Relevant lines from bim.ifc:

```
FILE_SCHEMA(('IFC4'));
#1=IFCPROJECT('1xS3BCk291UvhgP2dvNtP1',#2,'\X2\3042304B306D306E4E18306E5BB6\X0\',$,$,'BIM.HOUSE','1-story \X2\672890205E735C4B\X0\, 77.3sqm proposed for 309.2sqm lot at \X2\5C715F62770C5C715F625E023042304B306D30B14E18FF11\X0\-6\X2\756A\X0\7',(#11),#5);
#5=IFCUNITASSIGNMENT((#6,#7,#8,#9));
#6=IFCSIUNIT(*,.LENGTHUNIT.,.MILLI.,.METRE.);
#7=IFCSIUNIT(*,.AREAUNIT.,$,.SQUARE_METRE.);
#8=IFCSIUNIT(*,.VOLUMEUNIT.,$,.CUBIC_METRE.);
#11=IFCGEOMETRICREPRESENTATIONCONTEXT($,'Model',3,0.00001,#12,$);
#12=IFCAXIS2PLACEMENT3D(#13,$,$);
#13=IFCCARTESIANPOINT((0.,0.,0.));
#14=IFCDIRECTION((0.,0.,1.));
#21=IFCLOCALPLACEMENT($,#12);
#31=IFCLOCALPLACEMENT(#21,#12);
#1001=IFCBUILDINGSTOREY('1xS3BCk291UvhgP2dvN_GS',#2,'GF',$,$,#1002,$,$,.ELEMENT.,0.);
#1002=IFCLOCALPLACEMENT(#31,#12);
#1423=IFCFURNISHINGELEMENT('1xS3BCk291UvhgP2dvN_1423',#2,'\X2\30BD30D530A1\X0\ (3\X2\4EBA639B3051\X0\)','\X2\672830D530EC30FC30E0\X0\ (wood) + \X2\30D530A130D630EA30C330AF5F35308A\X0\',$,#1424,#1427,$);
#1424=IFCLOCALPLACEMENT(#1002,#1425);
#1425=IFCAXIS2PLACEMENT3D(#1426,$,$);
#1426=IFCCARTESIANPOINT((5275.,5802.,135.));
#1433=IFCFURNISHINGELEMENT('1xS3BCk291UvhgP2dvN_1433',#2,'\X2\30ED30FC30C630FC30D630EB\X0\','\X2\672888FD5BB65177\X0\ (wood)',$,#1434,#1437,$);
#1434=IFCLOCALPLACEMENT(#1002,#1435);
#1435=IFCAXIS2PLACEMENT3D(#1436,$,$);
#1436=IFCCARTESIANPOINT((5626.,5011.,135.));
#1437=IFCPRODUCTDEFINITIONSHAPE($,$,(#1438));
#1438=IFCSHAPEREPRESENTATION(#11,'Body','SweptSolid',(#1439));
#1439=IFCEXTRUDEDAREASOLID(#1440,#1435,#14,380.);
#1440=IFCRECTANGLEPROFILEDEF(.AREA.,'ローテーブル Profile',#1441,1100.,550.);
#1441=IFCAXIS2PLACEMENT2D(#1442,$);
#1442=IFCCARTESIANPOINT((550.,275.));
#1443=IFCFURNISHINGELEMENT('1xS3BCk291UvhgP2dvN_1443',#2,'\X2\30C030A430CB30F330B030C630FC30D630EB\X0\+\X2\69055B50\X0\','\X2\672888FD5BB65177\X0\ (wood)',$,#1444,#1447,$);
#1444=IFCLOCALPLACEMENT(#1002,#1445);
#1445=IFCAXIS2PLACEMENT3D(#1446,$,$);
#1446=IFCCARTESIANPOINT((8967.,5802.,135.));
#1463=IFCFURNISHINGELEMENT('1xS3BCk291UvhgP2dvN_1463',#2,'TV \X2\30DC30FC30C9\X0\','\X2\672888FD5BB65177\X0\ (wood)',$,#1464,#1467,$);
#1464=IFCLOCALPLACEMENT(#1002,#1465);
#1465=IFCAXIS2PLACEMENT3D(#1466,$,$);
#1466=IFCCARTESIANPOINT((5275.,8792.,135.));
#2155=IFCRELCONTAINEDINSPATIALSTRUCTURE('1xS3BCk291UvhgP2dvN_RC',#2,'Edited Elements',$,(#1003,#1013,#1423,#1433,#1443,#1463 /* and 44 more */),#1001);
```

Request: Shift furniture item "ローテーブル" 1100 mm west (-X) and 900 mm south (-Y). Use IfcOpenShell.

```python
import ifcopenshell
import ifcopenshell.api.geometry
import ifcopenshell.util.placement

model = ifcopenshell.open("bim.ifc")

item = model.by_guid("1xS3BCk291UvhgP2dvN_1433")
matrix = ifcopenshell.util.placement.get_local_placement(item.ObjectPlacement)
matrix[0, 3] -= 1100.0
matrix[1, 3] -= 900.0
ifcopenshell.api.geometry.edit_object_placement(model, product=item, matrix=matrix, is_si=False)

print(ifcopenshell.util.placement.get_local_placement(item.ObjectPlacement).round(3) + 0.0)

model.write("bim_edited.ifc")
```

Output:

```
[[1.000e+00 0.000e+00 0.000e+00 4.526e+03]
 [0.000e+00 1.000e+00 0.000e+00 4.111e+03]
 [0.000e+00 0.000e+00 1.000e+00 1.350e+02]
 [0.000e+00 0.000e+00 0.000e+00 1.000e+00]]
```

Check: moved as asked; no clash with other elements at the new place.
